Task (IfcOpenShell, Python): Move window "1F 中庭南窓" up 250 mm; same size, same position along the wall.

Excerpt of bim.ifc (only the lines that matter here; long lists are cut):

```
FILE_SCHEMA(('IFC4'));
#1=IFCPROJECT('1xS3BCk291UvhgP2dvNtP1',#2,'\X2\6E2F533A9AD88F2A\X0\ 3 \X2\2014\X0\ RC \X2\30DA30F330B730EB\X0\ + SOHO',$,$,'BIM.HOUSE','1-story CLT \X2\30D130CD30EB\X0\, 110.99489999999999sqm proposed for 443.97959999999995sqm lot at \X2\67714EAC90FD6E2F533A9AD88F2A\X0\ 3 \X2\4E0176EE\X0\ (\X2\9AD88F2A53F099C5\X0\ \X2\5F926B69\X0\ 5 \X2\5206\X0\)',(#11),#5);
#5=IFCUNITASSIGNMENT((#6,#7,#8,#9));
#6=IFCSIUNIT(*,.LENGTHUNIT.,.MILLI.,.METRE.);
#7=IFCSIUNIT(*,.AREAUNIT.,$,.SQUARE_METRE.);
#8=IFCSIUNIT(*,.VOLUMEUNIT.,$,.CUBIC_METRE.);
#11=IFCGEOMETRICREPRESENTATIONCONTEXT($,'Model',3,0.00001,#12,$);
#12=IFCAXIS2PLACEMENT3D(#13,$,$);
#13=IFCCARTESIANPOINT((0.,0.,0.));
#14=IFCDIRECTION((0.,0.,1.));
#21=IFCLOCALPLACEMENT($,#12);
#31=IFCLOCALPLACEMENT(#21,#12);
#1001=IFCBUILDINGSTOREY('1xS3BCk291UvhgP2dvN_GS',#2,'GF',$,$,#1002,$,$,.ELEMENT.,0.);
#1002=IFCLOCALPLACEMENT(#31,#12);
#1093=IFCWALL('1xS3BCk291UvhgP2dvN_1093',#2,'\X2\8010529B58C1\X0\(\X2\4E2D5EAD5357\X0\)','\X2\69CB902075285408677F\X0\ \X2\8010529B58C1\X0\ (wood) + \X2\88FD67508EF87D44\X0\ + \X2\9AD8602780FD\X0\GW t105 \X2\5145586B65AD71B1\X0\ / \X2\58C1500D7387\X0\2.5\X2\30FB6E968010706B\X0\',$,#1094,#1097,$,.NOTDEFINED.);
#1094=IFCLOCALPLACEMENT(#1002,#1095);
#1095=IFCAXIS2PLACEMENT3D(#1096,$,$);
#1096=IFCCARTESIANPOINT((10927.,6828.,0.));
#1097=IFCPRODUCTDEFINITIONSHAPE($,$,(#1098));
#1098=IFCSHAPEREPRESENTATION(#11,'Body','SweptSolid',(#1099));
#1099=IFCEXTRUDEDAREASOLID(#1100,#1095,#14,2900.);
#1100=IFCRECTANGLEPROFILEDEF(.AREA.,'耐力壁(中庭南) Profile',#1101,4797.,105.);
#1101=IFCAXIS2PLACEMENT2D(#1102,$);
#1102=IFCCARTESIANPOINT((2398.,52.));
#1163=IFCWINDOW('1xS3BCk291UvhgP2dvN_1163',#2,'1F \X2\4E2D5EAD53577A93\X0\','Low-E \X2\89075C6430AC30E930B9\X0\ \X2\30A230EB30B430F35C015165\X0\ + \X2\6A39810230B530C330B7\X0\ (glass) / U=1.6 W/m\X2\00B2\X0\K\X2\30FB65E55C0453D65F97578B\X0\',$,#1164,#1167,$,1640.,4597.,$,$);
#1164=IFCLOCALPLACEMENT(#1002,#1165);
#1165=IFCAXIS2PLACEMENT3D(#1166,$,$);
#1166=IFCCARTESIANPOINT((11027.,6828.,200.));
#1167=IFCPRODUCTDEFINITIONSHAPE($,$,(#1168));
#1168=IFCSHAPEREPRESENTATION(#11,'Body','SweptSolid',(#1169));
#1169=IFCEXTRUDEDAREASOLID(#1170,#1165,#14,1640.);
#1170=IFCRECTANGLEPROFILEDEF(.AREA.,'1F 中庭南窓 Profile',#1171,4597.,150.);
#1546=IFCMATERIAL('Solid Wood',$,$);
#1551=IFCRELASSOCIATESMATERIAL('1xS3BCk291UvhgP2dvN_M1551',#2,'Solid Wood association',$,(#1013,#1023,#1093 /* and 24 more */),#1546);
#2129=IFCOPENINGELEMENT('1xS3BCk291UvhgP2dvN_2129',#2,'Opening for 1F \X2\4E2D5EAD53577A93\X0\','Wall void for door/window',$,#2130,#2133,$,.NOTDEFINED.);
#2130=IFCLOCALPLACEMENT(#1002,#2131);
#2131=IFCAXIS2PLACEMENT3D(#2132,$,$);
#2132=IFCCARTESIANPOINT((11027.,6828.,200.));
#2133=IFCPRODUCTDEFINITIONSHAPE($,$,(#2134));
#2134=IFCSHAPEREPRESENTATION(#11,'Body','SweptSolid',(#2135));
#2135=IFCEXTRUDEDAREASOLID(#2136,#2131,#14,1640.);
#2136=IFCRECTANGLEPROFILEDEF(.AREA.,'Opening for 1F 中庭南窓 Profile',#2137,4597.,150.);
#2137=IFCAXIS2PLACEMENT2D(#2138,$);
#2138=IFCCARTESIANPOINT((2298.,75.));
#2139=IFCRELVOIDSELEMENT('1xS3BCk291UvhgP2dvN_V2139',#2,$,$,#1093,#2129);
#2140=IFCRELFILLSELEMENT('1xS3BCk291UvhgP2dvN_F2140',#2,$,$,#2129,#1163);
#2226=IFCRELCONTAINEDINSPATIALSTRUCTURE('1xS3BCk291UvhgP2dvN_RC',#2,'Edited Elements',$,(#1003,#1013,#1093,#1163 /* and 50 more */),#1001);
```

```python
import numpy as np
import ifcopenshell
import ifcopenshell.api.geometry
import ifcopenshell.util.placement
import ifcopenshell.util.unit

model = ifcopenshell.open("bim.ifc")
unit_scale = ifcopenshell.util.unit.calculate_unit_scale(model)

window = model.by_guid("1xS3BCk291UvhgP2dvN_1163")
opening = window.FillsVoids[0].RelatingOpeningElement
dz = 250.0

shift = np.array([0.0, 0.0, dz])
# The window is not placed relative to its opening, so move both.
for product in (opening, window):
    matrix = ifcopenshell.util.placement.get_local_placement(product.ObjectPlacement)
    matrix[:3, 3] += shift
    ifcopenshell.api.geometry.edit_object_placement(model, product=product, matrix=matrix, is_si=False)

print(f"moved by {dz * unit_scale:+.3f} m")

model.write("bim_updated.ifc")
```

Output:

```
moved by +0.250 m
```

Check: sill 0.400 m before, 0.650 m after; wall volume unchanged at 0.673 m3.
